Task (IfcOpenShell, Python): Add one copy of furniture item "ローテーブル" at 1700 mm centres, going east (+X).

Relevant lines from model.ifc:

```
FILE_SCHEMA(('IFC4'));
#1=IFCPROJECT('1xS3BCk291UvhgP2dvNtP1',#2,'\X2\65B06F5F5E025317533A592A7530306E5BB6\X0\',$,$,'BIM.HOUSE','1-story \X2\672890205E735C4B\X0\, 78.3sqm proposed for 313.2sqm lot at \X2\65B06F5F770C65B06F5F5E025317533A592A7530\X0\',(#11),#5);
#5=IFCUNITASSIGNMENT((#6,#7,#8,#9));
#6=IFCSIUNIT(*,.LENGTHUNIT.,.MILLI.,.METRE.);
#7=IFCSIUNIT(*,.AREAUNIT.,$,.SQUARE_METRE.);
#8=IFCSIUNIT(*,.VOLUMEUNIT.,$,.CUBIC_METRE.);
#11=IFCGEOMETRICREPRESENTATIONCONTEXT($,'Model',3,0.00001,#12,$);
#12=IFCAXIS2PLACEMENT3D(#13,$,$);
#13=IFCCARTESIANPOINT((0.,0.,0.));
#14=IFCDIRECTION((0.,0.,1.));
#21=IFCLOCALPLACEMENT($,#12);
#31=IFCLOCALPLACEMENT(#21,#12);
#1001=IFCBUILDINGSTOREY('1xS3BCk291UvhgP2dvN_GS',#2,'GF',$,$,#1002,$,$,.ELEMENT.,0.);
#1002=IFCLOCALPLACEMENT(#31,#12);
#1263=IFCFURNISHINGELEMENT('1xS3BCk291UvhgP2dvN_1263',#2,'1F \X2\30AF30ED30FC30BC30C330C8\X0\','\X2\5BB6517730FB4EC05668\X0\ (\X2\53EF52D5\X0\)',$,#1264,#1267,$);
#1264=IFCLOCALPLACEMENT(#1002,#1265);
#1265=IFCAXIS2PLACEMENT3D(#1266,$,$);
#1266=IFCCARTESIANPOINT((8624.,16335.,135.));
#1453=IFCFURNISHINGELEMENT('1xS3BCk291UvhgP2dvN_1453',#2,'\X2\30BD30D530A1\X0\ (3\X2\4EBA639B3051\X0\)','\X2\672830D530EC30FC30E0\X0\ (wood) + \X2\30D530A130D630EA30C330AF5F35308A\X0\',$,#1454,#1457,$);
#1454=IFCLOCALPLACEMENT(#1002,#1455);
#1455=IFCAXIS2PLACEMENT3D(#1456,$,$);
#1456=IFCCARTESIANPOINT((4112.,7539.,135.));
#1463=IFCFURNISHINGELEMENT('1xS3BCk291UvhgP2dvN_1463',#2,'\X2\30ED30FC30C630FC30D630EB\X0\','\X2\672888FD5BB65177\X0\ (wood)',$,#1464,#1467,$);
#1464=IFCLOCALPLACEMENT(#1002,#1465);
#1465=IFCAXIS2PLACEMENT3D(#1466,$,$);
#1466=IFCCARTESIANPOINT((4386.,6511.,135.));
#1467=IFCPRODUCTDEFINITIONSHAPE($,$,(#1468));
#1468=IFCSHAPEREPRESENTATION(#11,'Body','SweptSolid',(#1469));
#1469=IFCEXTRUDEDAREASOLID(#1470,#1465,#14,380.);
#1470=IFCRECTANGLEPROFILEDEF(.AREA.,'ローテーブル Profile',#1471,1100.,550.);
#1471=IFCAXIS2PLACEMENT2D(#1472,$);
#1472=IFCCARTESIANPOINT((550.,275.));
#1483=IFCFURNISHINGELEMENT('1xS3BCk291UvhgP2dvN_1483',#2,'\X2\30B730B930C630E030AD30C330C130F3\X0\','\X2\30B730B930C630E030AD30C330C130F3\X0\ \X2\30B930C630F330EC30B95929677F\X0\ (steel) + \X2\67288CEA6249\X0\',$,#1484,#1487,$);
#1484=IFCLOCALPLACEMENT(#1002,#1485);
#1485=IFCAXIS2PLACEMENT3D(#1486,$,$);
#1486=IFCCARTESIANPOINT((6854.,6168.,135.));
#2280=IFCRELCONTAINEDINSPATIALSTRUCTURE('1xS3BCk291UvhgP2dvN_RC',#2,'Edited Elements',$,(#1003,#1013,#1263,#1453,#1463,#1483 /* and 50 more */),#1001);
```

```python
import numpy as np
import ifcopenshell
import ifcopenshell.api.geometry
import ifcopenshell.api.root
import ifcopenshell.util.element
import ifcopenshell.util.placement

model = ifcopenshell.open("model.ifc")


def reuse_history(source, copy):
    """copy_class also copies each property set's owner history, people and application; keep the originals."""
    for rel in copy.IsDefinedBy:
        if rel.is_a("IfcRelDefinesByProperties") and (history := rel.RelatingPropertyDefinition.OwnerHistory):
            rel.RelatingPropertyDefinition.OwnerHistory = source.OwnerHistory
            ifcopenshell.util.element.remove_deep2(model, history)


source = model.by_guid("1xS3BCk291UvhgP2dvN_1463")
base = ifcopenshell.util.placement.get_local_placement(source.ObjectPlacement)
step = np.array([1.0, 0.0, 0.0]) * 1700.0

for i in range(1, 2):
    copy = ifcopenshell.api.root.copy_class(model, product=source)
    copy.Representation = ifcopenshell.util.element.copy_deep(
        model, source.Representation, exclude=["IfcGeometricRepresentationContext", "IfcRepresentationMap"]
    )
    reuse_history(source, copy)
    matrix = base.copy()
    matrix[:3, 3] += i * step
    print("added at", matrix[:3, 3].round(3) + 0.0)
    ifcopenshell.api.geometry.edit_object_placement(model, product=copy, matrix=matrix, is_si=False)

model.write("model_rev.ifc")
```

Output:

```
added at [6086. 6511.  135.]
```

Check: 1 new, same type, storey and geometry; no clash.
